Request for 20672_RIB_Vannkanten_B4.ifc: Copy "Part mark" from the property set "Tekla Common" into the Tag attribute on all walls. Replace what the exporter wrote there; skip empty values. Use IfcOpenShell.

First a look at what the model holds.

```python
import ifcopenshell
import ifcopenshell.util.element

model = ifcopenshell.open("20672_RIB_Vannkanten_B4.ifc")
print(model.schema)
walls = model.by_type("IfcWall")
print(len(walls), "walls")
for e in walls[:8]:
    source = ifcopenshell.util.element.get_pset(e, "Tekla Common", "Part mark")
    target = e.Tag
    print(e.id(), repr(source), repr(target), sep=" | ")
```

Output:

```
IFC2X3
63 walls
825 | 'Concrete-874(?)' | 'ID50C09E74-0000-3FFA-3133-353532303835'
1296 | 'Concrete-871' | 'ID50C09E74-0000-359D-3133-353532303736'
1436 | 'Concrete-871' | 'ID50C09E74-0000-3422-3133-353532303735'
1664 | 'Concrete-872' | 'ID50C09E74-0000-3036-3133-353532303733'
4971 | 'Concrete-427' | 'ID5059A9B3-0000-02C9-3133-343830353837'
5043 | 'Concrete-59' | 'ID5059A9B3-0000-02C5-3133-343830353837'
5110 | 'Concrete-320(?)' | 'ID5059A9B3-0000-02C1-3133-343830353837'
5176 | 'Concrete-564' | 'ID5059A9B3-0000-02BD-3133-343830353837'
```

```python
import ifcopenshell
import ifcopenshell.util.element

model = ifcopenshell.open("20672_RIB_Vannkanten_B4.ifc")

count = 0
for e in model.by_type("IfcWall"):
    value = ifcopenshell.util.element.get_pset(e, "Tekla Common", "Part mark")
    current = e.Tag
    if not value or not value.strip() or current == value:
        continue
    e.Tag = value
    count += 1

print(count, "walls updated")

model.write("20672_RIB_Vannkanten_B4_edited.ifc")
```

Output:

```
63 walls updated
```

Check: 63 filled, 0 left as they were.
